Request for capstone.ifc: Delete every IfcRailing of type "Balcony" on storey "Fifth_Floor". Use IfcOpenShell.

First a look at what the model holds.

```python
import ifcopenshell
import ifcopenshell.util.element

model = ifcopenshell.open("capstone.ifc")
print(model.schema)
storey = next(s for s in model.by_type("IfcBuildingStorey") if s.Name == "Fifth_Floor")
railings = [e for e in ifcopenshell.util.element.get_decomposition(storey) if e.is_a("IfcRailing")]
seen = {}
for e in railings:
    element_type = ifcopenshell.util.element.get_type(e)
    name = element_type.Name if element_type not in (None, e) else None
    seen[name] = seen.get(name, 0) + 1
for name, count in sorted(seen.items(), key=str):
    print(count, "x", name)
```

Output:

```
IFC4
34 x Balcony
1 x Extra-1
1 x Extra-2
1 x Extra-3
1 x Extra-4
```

```python
import ifcopenshell
import ifcopenshell.api.root
import ifcopenshell.util.element

model = ifcopenshell.open("capstone.ifc")

storey = next(s for s in model.by_type("IfcBuildingStorey") if s.Name == "Fifth_Floor")
railings = [e for e in ifcopenshell.util.element.get_decomposition(storey) if e.is_a("IfcRailing")]
targets = [e for e in railings if (t := ifcopenshell.util.element.get_type(e)) not in (None, e) and t.Name == "Balcony"]

for e in targets:
    ifcopenshell.api.root.remove_product(model, product=e)
print(len(targets), "removed")

model.write("capstone_edited.ifc")
```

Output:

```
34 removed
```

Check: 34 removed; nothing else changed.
